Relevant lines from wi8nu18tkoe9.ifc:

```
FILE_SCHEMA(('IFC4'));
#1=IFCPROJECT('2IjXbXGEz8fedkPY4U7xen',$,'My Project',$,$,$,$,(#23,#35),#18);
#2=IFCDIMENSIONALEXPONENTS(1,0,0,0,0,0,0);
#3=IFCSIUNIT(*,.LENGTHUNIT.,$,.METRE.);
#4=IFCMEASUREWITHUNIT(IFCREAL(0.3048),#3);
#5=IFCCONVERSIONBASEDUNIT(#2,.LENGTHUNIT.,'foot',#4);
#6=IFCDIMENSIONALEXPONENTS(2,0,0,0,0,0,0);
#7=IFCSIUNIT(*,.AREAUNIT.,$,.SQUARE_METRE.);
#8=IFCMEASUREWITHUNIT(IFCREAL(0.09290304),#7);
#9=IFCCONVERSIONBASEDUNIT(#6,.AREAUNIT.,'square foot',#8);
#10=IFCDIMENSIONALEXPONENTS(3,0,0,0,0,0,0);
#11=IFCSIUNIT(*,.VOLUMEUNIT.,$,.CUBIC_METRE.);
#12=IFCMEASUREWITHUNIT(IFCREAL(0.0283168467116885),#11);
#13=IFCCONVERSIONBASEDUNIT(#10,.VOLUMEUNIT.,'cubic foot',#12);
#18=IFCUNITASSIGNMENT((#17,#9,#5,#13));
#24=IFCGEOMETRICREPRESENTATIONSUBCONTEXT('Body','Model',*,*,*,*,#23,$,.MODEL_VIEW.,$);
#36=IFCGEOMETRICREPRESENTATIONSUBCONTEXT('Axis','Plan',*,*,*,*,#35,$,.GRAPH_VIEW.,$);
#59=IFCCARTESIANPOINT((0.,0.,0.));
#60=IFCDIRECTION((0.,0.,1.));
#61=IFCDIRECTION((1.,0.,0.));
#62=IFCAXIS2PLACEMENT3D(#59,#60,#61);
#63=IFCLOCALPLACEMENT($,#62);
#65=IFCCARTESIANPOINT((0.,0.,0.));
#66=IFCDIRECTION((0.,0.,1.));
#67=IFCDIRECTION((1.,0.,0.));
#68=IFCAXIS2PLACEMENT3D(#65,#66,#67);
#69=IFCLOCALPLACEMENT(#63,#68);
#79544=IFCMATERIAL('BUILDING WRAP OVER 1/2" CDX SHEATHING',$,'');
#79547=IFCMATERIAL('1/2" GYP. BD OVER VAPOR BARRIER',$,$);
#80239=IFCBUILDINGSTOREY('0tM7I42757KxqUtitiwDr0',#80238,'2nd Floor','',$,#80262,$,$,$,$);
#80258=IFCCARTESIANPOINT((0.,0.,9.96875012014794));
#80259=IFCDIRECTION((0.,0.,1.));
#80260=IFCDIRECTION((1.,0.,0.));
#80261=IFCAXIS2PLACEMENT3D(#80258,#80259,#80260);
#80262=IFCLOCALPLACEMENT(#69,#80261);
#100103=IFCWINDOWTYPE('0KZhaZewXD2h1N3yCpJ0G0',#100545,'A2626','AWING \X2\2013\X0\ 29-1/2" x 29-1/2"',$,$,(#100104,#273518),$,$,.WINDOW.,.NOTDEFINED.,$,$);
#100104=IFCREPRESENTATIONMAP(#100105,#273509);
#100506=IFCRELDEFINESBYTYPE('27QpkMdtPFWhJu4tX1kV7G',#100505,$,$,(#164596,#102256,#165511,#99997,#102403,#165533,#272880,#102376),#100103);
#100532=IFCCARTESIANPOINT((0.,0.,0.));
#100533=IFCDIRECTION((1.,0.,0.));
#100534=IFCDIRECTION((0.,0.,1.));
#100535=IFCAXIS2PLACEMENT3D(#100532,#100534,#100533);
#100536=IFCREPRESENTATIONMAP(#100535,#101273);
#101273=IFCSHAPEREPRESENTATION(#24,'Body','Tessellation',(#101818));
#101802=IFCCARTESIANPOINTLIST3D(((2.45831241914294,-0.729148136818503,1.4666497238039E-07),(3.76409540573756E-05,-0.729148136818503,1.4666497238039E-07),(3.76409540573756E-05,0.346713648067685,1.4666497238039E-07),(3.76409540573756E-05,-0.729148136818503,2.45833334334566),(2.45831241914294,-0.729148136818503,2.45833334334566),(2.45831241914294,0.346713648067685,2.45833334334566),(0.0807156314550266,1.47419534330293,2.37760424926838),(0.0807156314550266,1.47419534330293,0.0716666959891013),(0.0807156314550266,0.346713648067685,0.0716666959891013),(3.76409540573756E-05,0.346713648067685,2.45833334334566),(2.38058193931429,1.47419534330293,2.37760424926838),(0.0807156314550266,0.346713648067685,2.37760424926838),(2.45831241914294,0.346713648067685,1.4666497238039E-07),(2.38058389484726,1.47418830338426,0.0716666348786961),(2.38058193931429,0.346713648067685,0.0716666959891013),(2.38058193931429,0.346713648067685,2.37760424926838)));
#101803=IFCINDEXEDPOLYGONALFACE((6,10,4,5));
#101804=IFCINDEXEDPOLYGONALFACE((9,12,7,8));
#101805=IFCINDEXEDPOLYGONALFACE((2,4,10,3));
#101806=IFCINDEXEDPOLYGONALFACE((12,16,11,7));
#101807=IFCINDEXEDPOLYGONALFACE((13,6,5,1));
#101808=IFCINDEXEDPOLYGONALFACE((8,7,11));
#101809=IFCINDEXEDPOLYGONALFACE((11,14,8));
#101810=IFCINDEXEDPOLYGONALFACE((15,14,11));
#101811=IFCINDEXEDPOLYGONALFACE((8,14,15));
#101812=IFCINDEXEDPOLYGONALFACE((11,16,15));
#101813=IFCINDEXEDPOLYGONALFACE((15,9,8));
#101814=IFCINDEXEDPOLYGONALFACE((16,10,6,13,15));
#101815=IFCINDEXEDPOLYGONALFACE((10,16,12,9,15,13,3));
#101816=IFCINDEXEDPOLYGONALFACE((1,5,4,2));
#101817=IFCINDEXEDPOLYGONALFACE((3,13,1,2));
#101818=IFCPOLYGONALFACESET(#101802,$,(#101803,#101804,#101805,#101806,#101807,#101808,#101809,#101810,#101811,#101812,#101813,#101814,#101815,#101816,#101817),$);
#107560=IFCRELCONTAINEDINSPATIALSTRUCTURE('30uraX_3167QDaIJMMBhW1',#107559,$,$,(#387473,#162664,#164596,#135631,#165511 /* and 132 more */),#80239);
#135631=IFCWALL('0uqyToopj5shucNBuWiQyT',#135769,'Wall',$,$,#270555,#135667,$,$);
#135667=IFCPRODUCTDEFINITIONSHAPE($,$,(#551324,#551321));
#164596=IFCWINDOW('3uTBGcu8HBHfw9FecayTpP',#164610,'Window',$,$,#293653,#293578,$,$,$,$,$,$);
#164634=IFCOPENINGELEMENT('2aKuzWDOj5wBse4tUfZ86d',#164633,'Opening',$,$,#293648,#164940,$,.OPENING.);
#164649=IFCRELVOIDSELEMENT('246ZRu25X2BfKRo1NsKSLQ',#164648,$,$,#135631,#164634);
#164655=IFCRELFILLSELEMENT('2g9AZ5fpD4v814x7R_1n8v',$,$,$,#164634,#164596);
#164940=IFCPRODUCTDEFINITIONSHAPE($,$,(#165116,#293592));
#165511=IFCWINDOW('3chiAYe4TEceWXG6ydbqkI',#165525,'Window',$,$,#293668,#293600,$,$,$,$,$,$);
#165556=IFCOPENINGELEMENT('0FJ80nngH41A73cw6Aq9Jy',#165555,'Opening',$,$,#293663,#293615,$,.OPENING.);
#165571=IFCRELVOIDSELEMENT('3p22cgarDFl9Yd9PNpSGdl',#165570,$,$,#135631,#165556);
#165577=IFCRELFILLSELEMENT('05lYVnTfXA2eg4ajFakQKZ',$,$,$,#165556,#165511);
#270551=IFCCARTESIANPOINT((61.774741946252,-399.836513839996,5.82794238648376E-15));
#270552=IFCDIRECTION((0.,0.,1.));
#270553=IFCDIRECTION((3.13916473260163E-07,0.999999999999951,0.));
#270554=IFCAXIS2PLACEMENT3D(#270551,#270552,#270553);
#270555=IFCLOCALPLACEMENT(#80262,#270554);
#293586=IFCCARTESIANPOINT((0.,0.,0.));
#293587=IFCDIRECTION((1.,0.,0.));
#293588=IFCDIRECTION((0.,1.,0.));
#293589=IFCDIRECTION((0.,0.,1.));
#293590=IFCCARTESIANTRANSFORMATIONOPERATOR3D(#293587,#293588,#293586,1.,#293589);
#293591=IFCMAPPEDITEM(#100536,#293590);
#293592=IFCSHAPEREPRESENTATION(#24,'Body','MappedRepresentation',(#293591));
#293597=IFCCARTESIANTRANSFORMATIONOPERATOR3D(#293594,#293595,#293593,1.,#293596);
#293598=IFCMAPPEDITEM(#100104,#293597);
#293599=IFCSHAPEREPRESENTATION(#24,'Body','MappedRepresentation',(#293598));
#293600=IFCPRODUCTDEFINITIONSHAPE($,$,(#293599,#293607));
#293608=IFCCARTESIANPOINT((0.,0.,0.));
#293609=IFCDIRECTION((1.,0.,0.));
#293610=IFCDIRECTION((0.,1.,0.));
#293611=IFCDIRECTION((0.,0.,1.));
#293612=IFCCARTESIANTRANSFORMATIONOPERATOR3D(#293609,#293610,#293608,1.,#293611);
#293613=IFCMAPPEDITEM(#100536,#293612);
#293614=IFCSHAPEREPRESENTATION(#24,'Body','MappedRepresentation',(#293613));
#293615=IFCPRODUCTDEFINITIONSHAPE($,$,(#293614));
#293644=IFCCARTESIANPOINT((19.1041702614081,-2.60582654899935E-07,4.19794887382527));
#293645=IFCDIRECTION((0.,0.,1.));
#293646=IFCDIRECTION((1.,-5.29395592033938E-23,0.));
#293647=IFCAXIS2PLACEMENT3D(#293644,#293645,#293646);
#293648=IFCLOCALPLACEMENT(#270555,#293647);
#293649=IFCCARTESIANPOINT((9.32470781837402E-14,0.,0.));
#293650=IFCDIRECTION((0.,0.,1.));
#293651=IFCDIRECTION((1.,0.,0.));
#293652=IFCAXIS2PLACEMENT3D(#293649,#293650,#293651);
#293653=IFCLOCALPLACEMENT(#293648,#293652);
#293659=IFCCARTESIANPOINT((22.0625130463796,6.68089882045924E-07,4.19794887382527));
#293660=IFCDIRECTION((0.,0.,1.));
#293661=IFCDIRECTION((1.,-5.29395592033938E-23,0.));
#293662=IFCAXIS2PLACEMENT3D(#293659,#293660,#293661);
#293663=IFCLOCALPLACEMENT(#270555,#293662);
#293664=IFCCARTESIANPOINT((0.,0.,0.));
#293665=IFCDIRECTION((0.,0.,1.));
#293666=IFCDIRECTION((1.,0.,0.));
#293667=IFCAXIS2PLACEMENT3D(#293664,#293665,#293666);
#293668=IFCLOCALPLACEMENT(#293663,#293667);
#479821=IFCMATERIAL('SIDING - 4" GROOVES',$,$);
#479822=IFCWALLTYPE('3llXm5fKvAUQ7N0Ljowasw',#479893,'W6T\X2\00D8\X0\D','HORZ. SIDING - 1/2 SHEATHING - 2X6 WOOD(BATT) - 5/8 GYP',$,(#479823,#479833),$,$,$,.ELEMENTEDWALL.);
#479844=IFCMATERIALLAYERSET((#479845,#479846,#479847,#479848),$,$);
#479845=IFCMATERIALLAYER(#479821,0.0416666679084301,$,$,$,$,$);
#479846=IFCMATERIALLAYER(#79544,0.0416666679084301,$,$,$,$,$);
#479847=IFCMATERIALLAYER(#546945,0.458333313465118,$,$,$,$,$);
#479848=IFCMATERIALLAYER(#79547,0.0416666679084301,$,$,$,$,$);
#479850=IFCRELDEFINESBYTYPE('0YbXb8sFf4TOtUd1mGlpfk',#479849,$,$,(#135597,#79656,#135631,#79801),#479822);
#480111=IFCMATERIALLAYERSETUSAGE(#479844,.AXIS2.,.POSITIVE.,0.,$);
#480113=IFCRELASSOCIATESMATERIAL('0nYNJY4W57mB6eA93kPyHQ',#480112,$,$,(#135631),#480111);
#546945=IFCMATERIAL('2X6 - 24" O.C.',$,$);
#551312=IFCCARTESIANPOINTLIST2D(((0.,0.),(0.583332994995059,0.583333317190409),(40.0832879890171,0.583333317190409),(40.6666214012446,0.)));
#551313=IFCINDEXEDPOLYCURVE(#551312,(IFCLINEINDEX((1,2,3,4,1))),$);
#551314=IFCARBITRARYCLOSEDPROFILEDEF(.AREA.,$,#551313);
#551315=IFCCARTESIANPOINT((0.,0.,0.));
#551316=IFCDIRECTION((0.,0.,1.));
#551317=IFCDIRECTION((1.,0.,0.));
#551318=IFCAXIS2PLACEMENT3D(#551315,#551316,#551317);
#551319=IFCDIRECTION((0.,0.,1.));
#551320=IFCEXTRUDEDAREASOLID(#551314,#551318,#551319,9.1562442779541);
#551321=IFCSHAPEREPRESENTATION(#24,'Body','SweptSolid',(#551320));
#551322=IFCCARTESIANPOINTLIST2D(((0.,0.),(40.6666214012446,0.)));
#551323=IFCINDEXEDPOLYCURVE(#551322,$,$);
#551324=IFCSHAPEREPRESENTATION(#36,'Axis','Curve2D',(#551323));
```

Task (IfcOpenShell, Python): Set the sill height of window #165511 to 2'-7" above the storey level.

```python
import numpy as np
import ifcopenshell
import ifcopenshell.api.geometry
import ifcopenshell.geom
import ifcopenshell.util.element
import ifcopenshell.util.placement
import ifcopenshell.util.shape
import ifcopenshell.util.unit

model = ifcopenshell.open("wi8nu18tkoe9.ifc")
unit_scale = ifcopenshell.util.unit.calculate_unit_scale(model)

window = model.by_id(165511)
opening = window.FillsVoids[0].RelatingOpeningElement
storey = ifcopenshell.util.element.get_container(window, ifc_class="IfcBuildingStorey")
level = ifcopenshell.util.placement.get_local_placement(storey.ObjectPlacement)[2, 3]

# The opening's origin need not be at the sill, so measure its lowest point.
shape = ifcopenshell.geom.create_shape(ifcopenshell.geom.settings(), opening)
bottom = ifcopenshell.util.shape.get_shape_bottom_elevation(shape, shape.geometry) / unit_scale
dz = level + 31 * 0.0254 / unit_scale - bottom

shift = np.array([0.0, 0.0, dz])
# The window is placed relative to its opening, so it follows when the opening moves.
matrix = ifcopenshell.util.placement.get_local_placement(opening.ObjectPlacement)
matrix[:3, 3] += shift
ifcopenshell.api.geometry.edit_object_placement(
    model, product=opening, matrix=matrix, is_si=False, should_transform_children=True
)

print(f"moved by {dz * unit_scale:+.3f} m")

model.write("wi8nu18tkoe9_edited.ifc")
```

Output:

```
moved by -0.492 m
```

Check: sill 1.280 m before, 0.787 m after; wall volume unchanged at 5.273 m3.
